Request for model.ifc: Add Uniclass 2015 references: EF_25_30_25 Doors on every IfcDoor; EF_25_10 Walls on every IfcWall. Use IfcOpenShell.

First a look at what the model holds.

```python
import ifcopenshell

model = ifcopenshell.open("model.ifc")
print(model.schema)
print("classifications:", [c.Name for c in model.by_type("IfcClassification")])
for ifc_class in ("IfcDoor", "IfcRoof", "IfcStair", "IfcWall", "IfcWindow"):
    print(ifc_class, len(model.by_type(ifc_class)))
```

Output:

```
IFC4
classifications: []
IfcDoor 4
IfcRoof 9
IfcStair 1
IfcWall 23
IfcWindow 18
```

```python
import ifcopenshell
import ifcopenshell.api.classification

model = ifcopenshell.open("model.ifc")

system = ifcopenshell.api.classification.add_classification(model, classification="Uniclass 2015")

codes = {
    "IfcDoor": ("EF_25_30_25", "Doors"),
    "IfcWall": ("EF_25_10", "Walls"),
}
for ifc_class, (code, name) in codes.items():
    products = model.by_type(ifc_class)
    ifcopenshell.api.classification.add_reference(
        model, products=products, classification=system, identification=code, name=name
    )
    print(code, len(products))

model.write("model-out.ifc")
```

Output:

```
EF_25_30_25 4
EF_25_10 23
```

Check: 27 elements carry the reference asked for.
